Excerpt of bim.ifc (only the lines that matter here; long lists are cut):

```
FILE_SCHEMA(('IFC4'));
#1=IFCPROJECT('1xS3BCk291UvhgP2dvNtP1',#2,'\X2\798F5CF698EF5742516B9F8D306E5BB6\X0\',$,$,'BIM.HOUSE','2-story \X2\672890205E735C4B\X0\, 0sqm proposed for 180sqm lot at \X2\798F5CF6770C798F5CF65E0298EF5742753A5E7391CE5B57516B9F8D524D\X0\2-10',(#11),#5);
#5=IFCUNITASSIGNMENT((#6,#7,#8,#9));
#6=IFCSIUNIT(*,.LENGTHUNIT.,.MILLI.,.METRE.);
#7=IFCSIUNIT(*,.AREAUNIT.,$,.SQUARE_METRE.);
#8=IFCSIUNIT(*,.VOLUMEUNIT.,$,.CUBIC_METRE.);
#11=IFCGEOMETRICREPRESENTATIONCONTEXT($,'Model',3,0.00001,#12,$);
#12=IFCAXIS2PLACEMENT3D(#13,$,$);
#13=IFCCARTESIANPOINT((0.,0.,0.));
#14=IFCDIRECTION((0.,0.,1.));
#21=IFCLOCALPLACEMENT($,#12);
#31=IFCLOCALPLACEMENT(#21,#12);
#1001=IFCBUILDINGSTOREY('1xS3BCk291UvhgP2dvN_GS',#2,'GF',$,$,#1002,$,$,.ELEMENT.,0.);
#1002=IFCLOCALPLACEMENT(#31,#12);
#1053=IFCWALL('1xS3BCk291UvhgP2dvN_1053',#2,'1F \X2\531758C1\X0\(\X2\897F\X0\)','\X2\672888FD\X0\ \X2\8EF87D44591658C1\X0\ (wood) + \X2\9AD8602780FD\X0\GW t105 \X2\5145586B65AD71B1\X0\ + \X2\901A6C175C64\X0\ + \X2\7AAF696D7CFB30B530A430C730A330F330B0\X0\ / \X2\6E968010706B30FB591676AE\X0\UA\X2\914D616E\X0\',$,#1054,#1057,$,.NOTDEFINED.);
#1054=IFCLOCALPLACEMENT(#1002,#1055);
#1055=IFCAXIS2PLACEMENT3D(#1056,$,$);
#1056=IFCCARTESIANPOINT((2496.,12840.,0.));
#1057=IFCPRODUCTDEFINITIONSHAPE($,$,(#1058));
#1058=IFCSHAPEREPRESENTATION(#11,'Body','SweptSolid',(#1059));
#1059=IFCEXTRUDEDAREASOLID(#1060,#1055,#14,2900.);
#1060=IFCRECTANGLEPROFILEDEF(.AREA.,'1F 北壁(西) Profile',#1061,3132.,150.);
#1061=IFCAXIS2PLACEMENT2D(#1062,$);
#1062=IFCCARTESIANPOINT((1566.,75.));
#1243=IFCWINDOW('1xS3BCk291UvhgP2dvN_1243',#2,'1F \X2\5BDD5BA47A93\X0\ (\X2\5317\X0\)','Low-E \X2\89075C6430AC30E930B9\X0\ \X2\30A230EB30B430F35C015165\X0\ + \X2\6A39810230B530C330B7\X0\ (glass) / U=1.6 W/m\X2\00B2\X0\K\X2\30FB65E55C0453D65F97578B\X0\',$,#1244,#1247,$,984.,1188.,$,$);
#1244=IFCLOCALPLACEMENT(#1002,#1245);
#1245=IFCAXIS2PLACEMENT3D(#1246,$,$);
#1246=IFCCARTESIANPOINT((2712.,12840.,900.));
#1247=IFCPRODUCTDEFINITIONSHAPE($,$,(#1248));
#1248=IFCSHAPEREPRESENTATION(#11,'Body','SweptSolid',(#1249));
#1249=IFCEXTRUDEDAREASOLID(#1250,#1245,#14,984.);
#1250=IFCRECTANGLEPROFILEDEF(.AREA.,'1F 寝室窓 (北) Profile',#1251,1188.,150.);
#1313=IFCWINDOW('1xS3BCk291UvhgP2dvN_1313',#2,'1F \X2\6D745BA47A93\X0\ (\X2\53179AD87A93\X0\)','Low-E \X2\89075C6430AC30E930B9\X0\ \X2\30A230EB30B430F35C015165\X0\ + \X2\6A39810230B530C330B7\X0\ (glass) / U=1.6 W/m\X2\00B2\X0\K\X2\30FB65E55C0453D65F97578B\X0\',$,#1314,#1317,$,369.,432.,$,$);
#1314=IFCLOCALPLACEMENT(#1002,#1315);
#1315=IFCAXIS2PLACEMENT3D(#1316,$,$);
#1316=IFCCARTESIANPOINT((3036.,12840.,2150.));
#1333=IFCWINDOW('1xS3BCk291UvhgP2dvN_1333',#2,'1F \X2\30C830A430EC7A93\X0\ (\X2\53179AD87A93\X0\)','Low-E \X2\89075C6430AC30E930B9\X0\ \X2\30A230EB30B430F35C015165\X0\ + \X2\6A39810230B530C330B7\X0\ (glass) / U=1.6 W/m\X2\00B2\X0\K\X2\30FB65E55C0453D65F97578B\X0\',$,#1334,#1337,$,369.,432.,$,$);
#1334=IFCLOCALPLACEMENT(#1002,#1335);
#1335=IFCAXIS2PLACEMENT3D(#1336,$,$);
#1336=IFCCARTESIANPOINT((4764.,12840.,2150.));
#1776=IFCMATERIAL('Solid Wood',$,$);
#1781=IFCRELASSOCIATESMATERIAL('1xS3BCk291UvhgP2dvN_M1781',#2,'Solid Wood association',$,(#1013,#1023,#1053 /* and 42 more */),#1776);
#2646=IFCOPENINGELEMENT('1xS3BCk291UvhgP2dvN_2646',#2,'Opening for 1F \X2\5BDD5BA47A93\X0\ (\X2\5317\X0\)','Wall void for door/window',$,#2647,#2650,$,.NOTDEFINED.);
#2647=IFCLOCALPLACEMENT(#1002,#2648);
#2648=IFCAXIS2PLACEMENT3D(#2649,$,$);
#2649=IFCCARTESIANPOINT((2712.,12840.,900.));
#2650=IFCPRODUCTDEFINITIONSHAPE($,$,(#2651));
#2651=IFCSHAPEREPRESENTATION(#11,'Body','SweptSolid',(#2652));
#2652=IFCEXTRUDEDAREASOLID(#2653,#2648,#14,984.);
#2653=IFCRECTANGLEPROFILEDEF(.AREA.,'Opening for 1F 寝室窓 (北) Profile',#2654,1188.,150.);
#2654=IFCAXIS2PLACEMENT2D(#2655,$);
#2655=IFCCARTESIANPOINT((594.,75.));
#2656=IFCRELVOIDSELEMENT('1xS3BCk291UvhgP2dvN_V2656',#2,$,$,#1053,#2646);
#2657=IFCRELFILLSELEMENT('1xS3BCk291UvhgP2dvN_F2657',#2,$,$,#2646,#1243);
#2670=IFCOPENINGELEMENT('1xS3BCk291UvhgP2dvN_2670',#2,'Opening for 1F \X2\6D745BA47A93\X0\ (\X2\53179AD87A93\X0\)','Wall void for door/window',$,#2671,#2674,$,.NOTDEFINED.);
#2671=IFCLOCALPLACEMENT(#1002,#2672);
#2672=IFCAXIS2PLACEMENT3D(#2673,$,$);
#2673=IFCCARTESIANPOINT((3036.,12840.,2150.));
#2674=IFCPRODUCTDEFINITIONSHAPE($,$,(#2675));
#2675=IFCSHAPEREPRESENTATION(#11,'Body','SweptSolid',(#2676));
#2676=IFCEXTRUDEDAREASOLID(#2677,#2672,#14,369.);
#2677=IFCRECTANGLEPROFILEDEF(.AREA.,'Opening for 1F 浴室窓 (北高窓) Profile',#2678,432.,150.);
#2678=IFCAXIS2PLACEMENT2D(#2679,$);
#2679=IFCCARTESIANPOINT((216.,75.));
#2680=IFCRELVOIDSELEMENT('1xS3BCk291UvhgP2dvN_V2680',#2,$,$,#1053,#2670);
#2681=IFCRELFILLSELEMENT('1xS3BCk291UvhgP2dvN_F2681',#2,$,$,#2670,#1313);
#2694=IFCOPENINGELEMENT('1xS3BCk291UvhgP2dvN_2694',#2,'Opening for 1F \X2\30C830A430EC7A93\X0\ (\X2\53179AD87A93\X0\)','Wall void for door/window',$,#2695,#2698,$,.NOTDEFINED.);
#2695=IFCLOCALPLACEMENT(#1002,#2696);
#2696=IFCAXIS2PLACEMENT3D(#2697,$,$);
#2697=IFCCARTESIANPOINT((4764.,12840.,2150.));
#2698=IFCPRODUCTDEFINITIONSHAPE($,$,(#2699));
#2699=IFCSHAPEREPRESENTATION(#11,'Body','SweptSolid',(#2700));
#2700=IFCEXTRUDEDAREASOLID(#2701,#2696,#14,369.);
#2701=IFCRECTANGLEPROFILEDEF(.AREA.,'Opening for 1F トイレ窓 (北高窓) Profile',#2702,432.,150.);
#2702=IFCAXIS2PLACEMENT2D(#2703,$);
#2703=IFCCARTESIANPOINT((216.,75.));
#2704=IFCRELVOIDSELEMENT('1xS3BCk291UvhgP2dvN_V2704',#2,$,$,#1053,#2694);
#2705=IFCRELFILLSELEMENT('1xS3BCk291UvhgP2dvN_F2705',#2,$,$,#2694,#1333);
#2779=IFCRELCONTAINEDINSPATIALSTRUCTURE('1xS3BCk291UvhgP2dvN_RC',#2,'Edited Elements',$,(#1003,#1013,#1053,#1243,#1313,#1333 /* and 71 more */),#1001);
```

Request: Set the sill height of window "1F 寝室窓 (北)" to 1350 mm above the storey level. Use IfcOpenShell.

```python
import numpy as np
import ifcopenshell
import ifcopenshell.api.geometry
import ifcopenshell.geom
import ifcopenshell.util.element
import ifcopenshell.util.placement
import ifcopenshell.util.shape
import ifcopenshell.util.unit

model = ifcopenshell.open("bim.ifc")
unit_scale = ifcopenshell.util.unit.calculate_unit_scale(model)

window = model.by_id(1243)
opening = window.FillsVoids[0].RelatingOpeningElement
storey = ifcopenshell.util.element.get_container(window, ifc_class="IfcBuildingStorey")
level = ifcopenshell.util.placement.get_local_placement(storey.ObjectPlacement)[2, 3]

# The opening's origin need not be at the sill, so measure its lowest point.
shape = ifcopenshell.geom.create_shape(ifcopenshell.geom.settings(), opening)
bottom = ifcopenshell.util.shape.get_shape_bottom_elevation(shape, shape.geometry) / unit_scale
dz = level + 1350.0 - bottom

shift = np.array([0.0, 0.0, dz])
# The window is not placed relative to its opening, so move both.
for product in (opening, window):
    matrix = ifcopenshell.util.placement.get_local_placement(product.ObjectPlacement)
    matrix[:3, 3] += shift
    ifcopenshell.api.geometry.edit_object_placement(model, product=product, matrix=matrix, is_si=False)

print(f"moved by {dz * unit_scale:+.3f} m")

model.write("bim_v2.ifc")
```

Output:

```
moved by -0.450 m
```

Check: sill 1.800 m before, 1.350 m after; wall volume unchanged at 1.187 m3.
